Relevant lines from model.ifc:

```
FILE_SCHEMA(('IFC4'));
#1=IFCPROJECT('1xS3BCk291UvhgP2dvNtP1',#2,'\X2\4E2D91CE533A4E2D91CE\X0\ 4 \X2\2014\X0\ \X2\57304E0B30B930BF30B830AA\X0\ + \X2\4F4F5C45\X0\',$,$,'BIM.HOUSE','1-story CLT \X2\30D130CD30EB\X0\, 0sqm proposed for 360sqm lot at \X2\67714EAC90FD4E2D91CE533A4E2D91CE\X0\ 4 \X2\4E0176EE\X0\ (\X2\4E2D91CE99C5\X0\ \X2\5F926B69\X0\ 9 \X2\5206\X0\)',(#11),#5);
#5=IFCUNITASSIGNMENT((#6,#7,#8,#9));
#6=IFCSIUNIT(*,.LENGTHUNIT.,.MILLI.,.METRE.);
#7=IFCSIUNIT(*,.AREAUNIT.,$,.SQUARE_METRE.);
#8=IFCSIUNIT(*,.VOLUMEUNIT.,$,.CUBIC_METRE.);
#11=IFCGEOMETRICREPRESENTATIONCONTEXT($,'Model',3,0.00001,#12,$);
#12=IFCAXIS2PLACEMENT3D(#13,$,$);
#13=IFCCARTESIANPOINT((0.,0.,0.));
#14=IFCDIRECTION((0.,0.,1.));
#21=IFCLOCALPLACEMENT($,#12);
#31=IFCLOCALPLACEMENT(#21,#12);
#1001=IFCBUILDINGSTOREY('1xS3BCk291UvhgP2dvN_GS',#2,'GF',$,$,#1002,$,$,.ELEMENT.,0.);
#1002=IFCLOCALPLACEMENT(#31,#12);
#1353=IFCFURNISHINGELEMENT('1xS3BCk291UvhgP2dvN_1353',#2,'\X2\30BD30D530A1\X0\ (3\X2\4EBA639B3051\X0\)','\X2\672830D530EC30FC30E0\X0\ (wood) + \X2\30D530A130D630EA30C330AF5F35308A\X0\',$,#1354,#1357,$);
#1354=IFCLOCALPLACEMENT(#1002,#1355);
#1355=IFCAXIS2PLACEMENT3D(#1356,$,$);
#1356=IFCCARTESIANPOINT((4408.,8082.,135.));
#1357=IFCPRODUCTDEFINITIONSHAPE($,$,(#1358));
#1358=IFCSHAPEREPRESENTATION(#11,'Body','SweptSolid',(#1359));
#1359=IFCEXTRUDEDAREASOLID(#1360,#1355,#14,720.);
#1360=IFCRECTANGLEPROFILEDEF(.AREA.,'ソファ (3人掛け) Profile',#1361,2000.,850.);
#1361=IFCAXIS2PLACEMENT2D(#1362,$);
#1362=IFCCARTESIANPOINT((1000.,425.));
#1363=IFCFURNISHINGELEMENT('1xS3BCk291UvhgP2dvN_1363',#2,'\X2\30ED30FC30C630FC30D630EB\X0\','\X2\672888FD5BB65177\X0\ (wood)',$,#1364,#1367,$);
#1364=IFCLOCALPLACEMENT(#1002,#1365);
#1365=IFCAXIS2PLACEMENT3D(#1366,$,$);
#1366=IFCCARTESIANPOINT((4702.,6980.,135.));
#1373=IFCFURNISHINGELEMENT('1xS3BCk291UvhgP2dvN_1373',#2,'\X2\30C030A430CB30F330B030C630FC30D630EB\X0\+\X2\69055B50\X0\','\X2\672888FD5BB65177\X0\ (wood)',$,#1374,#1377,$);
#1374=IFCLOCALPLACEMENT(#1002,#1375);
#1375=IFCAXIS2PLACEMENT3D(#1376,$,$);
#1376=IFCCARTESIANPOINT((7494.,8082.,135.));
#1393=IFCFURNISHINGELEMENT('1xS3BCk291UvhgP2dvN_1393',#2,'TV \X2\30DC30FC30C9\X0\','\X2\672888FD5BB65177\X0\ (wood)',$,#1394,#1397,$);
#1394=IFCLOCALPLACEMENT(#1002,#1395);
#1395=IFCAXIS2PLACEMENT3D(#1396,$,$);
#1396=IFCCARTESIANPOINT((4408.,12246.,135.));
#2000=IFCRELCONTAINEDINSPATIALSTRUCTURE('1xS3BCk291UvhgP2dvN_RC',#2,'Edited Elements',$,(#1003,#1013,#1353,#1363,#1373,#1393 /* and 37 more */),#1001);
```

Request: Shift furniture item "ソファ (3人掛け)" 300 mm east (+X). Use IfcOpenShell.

```python
import ifcopenshell
import ifcopenshell.api.geometry
import ifcopenshell.util.placement

model = ifcopenshell.open("model.ifc")

item = model.by_guid("1xS3BCk291UvhgP2dvN_1353")
matrix = ifcopenshell.util.placement.get_local_placement(item.ObjectPlacement)
matrix[0, 3] += 300.0
ifcopenshell.api.geometry.edit_object_placement(model, product=item, matrix=matrix, is_si=False)

print(ifcopenshell.util.placement.get_local_placement(item.ObjectPlacement).round(3) + 0.0)

model.write("model_rev.ifc")
```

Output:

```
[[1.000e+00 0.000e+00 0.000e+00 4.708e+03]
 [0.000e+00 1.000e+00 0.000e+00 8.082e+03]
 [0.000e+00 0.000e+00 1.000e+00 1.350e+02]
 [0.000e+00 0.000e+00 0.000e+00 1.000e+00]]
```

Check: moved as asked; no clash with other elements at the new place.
